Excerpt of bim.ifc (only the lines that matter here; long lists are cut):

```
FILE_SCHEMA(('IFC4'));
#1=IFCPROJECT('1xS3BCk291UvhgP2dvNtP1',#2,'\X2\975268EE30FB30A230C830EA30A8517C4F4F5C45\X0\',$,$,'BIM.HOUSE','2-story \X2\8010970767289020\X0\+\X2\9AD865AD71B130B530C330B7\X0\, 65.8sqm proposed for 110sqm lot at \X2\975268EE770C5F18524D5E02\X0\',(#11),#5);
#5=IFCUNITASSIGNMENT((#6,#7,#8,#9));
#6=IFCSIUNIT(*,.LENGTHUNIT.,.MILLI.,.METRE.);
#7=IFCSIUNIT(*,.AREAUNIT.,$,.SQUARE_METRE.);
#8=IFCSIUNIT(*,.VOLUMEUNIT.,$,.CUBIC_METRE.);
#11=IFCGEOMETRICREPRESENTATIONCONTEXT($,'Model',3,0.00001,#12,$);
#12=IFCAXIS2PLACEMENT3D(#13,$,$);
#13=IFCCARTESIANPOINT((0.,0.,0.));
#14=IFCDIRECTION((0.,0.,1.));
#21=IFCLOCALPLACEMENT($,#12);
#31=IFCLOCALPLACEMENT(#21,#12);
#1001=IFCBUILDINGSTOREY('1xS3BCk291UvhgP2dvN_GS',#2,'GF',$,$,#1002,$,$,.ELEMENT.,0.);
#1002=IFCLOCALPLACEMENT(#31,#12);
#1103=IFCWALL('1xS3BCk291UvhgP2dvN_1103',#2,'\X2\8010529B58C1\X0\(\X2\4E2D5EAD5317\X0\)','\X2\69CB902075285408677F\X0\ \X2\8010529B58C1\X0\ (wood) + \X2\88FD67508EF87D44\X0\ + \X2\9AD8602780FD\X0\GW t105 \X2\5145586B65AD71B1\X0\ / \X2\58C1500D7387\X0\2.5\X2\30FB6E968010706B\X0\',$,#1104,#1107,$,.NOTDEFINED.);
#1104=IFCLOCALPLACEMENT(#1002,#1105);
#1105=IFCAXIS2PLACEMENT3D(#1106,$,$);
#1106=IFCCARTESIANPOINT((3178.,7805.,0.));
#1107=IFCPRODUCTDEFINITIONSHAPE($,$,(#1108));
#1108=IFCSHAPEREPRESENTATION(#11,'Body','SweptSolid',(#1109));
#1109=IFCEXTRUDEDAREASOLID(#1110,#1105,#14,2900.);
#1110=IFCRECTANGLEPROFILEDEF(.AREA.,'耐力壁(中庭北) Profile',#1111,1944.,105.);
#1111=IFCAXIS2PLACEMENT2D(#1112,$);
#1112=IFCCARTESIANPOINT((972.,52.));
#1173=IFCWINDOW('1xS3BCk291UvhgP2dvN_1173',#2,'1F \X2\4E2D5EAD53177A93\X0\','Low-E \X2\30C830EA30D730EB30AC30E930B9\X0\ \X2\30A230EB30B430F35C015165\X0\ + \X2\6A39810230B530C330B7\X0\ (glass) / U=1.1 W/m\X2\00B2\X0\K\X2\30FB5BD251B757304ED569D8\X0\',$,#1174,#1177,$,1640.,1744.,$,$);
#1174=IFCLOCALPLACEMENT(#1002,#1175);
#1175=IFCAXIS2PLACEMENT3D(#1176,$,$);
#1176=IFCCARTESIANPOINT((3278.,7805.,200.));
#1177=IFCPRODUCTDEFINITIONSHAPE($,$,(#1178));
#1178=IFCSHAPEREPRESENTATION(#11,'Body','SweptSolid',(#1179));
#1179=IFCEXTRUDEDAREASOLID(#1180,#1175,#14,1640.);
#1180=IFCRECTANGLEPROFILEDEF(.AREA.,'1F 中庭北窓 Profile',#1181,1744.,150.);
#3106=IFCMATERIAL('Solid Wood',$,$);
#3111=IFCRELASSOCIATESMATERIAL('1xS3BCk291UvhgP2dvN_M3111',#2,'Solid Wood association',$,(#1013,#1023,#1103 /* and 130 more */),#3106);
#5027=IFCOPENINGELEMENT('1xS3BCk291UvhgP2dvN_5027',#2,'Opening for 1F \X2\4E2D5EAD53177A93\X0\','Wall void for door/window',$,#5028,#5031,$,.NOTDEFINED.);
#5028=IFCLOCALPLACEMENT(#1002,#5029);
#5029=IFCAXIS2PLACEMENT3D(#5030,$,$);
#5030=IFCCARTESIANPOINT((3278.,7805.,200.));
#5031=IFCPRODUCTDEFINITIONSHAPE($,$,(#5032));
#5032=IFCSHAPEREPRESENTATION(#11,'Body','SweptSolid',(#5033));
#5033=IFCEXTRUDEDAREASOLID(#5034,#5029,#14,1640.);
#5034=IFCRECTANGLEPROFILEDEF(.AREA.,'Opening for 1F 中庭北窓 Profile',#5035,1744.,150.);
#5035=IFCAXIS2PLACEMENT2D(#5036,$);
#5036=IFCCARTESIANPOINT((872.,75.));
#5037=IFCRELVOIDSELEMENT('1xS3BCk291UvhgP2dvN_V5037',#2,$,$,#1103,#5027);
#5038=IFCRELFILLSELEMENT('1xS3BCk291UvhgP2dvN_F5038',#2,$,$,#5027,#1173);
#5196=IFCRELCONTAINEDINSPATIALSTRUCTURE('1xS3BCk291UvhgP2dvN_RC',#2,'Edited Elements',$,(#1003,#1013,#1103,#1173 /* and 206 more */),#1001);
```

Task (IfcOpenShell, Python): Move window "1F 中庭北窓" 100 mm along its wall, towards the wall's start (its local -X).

```python
import ifcopenshell
import ifcopenshell.api.geometry
import ifcopenshell.util.placement

model = ifcopenshell.open("bim.ifc")

window = model.by_id(1173)
opening = window.FillsVoids[0].RelatingOpeningElement
wall = opening.VoidsElements[0].RelatingBuildingElement

wall_matrix = ifcopenshell.util.placement.get_local_placement(wall.ObjectPlacement)
shift = wall_matrix[:3, 0] * -100.0
before = ifcopenshell.util.placement.get_local_placement(window.ObjectPlacement)[:3, 3].copy()

# The window is not placed relative to its opening, so move both.
for product in (opening, window):
    matrix = ifcopenshell.util.placement.get_local_placement(product.ObjectPlacement)
    matrix[:3, 3] += shift
    ifcopenshell.api.geometry.edit_object_placement(model, product=product, matrix=matrix, is_si=False)

after = ifcopenshell.util.placement.get_local_placement(window.ObjectPlacement)[:3, 3]
print("window moved by", (after - before).round(3) + 0.0)

model.write("bim_updated.ifc")
```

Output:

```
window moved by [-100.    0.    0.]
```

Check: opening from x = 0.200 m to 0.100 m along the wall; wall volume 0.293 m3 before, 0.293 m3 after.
